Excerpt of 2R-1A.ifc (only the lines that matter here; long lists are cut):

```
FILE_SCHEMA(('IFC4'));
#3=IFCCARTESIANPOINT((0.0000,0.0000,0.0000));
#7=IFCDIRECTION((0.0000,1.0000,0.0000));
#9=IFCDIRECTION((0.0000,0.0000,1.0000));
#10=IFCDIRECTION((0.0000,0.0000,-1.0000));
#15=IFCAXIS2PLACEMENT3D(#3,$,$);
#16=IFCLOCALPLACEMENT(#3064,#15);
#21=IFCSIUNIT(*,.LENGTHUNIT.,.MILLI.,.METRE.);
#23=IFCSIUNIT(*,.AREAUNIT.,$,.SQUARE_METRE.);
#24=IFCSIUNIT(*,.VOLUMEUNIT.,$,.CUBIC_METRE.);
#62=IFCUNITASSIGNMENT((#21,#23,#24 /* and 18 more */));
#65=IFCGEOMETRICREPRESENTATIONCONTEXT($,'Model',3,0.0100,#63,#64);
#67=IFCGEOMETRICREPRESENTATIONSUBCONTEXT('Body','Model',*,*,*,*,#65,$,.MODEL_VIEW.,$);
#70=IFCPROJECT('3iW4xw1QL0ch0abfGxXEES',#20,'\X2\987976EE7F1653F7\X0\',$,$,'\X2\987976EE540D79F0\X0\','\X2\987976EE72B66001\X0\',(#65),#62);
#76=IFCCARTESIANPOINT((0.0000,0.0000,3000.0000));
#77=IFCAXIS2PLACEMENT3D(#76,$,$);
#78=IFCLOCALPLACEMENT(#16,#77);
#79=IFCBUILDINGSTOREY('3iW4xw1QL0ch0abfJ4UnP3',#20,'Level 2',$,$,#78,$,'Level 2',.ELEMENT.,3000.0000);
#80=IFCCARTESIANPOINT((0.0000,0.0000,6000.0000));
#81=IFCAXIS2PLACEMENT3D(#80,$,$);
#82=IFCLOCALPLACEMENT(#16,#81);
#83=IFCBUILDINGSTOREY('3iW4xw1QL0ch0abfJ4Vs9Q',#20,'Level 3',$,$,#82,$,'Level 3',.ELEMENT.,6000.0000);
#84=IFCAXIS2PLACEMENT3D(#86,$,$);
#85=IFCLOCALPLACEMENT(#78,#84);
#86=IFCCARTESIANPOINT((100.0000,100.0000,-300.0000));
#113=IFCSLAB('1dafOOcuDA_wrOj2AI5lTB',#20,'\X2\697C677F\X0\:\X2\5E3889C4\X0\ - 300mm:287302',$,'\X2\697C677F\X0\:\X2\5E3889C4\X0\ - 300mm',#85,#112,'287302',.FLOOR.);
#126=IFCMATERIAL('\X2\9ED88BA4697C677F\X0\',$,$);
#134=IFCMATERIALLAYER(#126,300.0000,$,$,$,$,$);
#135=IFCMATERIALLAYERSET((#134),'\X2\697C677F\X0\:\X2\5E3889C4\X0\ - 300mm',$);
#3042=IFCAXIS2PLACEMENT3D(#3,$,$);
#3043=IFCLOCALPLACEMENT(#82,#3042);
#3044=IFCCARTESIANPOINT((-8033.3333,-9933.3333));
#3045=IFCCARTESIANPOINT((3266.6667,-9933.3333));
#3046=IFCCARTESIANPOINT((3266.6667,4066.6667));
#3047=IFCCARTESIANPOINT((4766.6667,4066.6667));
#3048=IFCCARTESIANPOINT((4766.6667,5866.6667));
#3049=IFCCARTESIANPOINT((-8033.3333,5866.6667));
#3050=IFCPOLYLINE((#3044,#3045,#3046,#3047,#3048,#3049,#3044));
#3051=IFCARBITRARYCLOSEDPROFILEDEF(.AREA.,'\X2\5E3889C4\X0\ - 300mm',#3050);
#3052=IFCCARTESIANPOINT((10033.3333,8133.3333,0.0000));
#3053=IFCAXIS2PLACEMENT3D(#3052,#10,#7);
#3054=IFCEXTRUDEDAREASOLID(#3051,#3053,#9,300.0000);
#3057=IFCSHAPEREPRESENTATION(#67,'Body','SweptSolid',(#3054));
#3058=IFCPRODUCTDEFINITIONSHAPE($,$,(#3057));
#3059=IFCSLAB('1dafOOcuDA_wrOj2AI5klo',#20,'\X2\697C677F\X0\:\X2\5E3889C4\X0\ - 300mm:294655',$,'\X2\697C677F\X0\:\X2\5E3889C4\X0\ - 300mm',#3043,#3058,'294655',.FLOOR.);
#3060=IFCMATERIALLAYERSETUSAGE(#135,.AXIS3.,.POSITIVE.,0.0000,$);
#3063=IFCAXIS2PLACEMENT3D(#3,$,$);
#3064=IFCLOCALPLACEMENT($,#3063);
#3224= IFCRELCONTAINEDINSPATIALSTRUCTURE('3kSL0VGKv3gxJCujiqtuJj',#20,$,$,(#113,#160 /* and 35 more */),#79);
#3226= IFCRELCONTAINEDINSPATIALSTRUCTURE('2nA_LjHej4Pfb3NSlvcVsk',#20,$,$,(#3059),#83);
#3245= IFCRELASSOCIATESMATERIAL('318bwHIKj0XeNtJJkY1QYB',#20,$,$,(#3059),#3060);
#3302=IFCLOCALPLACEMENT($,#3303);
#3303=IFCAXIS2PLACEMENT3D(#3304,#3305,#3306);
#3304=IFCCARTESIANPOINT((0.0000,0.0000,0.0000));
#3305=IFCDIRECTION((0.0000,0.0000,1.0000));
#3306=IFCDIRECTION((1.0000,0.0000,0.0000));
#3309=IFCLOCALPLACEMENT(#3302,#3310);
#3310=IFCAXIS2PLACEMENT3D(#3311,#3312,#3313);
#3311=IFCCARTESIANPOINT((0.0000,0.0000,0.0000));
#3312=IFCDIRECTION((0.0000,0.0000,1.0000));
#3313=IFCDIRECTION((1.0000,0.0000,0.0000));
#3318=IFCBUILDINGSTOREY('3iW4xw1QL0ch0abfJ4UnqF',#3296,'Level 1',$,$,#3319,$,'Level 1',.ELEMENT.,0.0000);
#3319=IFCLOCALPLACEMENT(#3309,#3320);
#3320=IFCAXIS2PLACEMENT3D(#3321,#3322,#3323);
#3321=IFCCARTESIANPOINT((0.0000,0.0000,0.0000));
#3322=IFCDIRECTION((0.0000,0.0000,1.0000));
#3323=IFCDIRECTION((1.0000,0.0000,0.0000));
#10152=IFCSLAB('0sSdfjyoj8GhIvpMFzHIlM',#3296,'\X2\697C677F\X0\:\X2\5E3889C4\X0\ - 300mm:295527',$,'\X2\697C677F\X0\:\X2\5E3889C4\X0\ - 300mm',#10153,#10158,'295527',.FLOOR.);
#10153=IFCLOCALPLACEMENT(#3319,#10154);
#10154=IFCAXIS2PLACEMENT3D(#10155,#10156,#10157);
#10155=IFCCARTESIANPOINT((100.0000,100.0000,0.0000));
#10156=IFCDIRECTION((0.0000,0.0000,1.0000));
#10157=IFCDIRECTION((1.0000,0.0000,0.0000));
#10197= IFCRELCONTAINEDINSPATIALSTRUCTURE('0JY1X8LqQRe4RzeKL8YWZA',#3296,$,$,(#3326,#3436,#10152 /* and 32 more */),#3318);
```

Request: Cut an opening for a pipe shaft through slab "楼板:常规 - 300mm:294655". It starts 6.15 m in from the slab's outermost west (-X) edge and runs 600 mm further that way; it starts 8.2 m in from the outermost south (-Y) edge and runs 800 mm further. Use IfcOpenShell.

```python
import numpy as np
import ifcopenshell
import ifcopenshell.api.feature
import ifcopenshell.api.geometry
import ifcopenshell.api.root
import ifcopenshell.geom
import ifcopenshell.util.placement
import ifcopenshell.util.representation
import ifcopenshell.util.shape
import ifcopenshell.util.unit

model = ifcopenshell.open("2R-1A.ifc")
unit_scale = ifcopenshell.util.unit.calculate_unit_scale(model)
settings = ifcopenshell.geom.settings()


def volume(element):
    """Net volume in cubic metres, openings subtracted."""
    shape = ifcopenshell.geom.create_shape(settings, element)
    return ifcopenshell.util.shape.get_volume(shape.geometry)


slab = model.by_id(3059)
before = volume(slab)

# Extent in the slab's own axes, in metres. The edges named are its -X and -Y sides.
slab_shape = ifcopenshell.geom.create_shape(settings, slab)
vertices = ifcopenshell.util.shape.get_vertices(slab_shape.geometry)
x_min, y_min, bottom = vertices.min(axis=0)
top = vertices[:, 2].max()

opening = ifcopenshell.api.root.create_entity(model, ifc_class="IfcOpeningElement", name="Pipe shaft opening", predefined_type="OPENING")
context = ifcopenshell.util.representation.get_context(model, "Model", "Body", "MODEL_VIEW")
width, depth = 0.6, 0.8
outline = [(0.0, 0.0), (width, 0.0), (width, depth), (0.0, depth), (0.0, 0.0)]
# Overshoot both faces by 50 mm so the cut is clean.
shape = ifcopenshell.api.geometry.add_slab_representation(
    model, context=context, depth=top - bottom + 0.1, polyline=outline
)
ifcopenshell.api.geometry.assign_representation(model, product=opening, representation=shape)

matrix = ifcopenshell.util.placement.get_local_placement(slab.ObjectPlacement)
matrix[:, 3] = matrix @ np.append(np.array([x_min + 6.15, y_min + 8.2, bottom - 0.05]) / unit_scale, 1.0)
ifcopenshell.api.geometry.edit_object_placement(model, product=opening, matrix=matrix, is_si=False)
ifcopenshell.api.feature.add_feature(model, feature=opening, element=slab)

after = volume(slab)

print(f"slab volume {before:.3f} -> {after:.3f} m3")

model.write("2R-1A_edited.ifc")
```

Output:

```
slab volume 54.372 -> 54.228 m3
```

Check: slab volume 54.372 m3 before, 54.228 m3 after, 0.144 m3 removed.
